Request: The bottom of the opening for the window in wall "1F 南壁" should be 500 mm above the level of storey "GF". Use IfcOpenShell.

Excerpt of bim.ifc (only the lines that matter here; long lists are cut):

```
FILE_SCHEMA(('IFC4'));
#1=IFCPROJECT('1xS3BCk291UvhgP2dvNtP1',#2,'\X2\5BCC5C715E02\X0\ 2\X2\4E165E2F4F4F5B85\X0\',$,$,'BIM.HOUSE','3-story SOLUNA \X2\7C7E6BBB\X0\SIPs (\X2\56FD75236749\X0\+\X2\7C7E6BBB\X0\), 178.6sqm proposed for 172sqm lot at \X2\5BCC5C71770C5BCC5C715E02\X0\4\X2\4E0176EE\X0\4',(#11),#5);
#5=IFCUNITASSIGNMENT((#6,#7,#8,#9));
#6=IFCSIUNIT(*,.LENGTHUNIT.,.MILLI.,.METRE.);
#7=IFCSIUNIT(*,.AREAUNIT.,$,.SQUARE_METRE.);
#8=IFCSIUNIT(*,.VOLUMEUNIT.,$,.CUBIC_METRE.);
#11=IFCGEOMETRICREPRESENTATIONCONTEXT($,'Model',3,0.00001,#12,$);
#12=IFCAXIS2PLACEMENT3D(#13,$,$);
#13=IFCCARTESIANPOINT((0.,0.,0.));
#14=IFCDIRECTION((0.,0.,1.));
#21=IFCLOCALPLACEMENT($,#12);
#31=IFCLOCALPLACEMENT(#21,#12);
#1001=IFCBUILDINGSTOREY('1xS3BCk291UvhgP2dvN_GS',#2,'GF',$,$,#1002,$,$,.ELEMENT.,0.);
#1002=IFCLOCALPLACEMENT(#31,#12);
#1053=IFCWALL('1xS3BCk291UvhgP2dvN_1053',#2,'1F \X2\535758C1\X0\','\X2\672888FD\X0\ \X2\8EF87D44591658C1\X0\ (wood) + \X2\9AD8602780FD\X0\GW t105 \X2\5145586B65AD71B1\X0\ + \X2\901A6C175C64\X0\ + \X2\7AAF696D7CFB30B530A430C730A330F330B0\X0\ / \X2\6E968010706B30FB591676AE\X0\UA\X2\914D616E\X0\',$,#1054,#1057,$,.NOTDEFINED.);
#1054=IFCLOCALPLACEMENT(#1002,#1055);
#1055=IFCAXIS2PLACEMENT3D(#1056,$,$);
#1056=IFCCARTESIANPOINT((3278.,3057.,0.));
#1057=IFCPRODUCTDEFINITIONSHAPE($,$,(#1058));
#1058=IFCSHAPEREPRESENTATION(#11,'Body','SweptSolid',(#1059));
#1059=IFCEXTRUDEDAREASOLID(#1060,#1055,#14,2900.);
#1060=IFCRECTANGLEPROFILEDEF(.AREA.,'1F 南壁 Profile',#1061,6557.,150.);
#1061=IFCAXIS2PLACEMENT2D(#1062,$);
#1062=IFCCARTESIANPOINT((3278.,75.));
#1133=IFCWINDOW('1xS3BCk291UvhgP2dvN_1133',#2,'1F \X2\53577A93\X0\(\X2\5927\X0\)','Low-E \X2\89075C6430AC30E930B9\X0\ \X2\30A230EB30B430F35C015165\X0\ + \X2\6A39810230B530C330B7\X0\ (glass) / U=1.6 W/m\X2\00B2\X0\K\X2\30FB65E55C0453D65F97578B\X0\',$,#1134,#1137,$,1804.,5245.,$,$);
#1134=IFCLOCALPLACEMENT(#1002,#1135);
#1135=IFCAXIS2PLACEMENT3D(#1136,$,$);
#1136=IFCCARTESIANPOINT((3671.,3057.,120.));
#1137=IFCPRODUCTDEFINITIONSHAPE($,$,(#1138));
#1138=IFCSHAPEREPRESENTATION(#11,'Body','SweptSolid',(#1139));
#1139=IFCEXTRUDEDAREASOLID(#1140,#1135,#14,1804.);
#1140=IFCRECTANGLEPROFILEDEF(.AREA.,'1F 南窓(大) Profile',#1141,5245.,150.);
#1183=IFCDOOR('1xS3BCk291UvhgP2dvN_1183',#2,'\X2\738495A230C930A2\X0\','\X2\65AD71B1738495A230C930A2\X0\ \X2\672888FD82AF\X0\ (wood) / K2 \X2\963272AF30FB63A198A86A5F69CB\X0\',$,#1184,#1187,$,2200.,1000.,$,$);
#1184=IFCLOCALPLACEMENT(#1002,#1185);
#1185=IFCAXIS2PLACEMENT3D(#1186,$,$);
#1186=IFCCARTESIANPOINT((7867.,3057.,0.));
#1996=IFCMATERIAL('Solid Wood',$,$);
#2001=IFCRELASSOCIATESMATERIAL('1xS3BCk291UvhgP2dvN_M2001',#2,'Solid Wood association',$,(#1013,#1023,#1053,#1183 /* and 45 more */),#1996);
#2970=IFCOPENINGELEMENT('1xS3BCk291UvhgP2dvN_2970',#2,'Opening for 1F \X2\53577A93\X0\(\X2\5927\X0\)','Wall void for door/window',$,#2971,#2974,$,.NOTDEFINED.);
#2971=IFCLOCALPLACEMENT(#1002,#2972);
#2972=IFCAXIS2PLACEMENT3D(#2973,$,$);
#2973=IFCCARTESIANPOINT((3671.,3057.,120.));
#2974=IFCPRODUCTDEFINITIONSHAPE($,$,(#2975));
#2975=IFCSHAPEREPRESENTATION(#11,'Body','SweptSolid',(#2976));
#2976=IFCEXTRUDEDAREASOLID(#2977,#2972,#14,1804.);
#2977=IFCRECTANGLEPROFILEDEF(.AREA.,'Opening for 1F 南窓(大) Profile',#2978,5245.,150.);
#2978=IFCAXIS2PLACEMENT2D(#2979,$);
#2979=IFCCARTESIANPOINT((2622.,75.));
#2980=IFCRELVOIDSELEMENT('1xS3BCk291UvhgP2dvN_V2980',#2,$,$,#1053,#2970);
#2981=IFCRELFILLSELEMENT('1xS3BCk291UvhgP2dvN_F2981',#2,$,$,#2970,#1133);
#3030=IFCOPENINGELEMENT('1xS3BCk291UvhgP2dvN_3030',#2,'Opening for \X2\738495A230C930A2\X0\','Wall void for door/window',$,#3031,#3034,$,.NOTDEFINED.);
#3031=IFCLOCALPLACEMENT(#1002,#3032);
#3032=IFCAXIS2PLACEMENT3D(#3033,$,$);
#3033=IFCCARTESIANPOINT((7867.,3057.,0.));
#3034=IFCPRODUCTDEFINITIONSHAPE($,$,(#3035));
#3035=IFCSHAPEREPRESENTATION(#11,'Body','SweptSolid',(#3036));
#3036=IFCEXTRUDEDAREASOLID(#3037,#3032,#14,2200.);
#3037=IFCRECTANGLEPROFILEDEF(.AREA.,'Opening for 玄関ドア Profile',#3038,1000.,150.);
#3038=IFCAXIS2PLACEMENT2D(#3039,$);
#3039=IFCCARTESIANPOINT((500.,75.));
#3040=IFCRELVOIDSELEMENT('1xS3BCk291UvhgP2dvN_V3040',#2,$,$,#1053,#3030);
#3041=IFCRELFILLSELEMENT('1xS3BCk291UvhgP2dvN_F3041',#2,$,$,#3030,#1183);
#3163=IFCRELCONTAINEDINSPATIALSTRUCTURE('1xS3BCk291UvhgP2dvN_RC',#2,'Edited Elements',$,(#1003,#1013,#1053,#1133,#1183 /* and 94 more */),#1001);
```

```python
import numpy as np
import ifcopenshell
import ifcopenshell.api.geometry
import ifcopenshell.geom
import ifcopenshell.util.element
import ifcopenshell.util.placement
import ifcopenshell.util.shape
import ifcopenshell.util.unit

model = ifcopenshell.open("bim.ifc")
unit_scale = ifcopenshell.util.unit.calculate_unit_scale(model)

window = model.by_guid("1xS3BCk291UvhgP2dvN_1133")
opening = window.FillsVoids[0].RelatingOpeningElement
storey = ifcopenshell.util.element.get_container(window, ifc_class="IfcBuildingStorey")
level = ifcopenshell.util.placement.get_local_placement(storey.ObjectPlacement)[2, 3]

# The opening's origin need not be at the sill, so measure its lowest point.
shape = ifcopenshell.geom.create_shape(ifcopenshell.geom.settings(), opening)
bottom = ifcopenshell.util.shape.get_shape_bottom_elevation(shape, shape.geometry) / unit_scale
dz = level + 0.5 / unit_scale - bottom

shift = np.array([0.0, 0.0, dz])
# The window is not placed relative to its opening, so move both.
for product in (opening, window):
    matrix = ifcopenshell.util.placement.get_local_placement(product.ObjectPlacement)
    matrix[:3, 3] += shift
    ifcopenshell.api.geometry.edit_object_placement(model, product=product, matrix=matrix, is_si=False)

print(f"moved by {dz * unit_scale:+.3f} m")

model.write("bim_v2.ifc")
```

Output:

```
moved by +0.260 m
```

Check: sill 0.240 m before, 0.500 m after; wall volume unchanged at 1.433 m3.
